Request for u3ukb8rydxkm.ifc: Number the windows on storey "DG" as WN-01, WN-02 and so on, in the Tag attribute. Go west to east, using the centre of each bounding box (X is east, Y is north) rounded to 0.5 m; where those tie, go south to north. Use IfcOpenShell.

First a look at what the model holds.

```python
import ifcopenshell
import ifcopenshell.util.element
import ifcopenshell.util.placement

model = ifcopenshell.open("u3ukb8rydxkm.ifc")
print(model.schema)
storey = next(s for s in model.by_type("IfcBuildingStorey") if s.Name == "DG")
windows = [e for e in ifcopenshell.util.element.get_decomposition(storey) if e.is_a("IfcWindow")]
for e in sorted(windows, key=lambda e: e.id()):
    origin = ifcopenshell.util.placement.get_local_placement(e.ObjectPlacement)[:3, 3]
    print(e.id(), e.Tag, e.Name, origin.round(2) + 0.0, sep=" | ")
```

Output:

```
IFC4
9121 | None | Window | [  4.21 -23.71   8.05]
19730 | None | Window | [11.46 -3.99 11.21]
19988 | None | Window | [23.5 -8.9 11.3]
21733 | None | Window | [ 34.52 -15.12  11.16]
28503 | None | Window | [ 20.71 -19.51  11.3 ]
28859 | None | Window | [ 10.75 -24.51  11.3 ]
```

```python
import ifcopenshell
import ifcopenshell.geom
import ifcopenshell.util.element
import ifcopenshell.util.shape

model = ifcopenshell.open("u3ukb8rydxkm.ifc")
settings = ifcopenshell.geom.settings()
settings.set("use-world-coords", True)


def centre(element):
    shape = ifcopenshell.geom.create_shape(settings, element)
    return ifcopenshell.util.shape.get_bbox_centroid(shape.geometry)


storey = next(s for s in model.by_type("IfcBuildingStorey") if s.Name == "DG")
windows = [e for e in ifcopenshell.util.element.get_decomposition(storey) if e.is_a("IfcWindow")]

# Insertion points can sit at a corner or the storey origin, so sort by the geometry (in metres).
centres = {e: centre(e) for e in windows}
windows.sort(key=lambda e: (round(centres[e][0] / 0.5), centres[e][1]))

for i, e in enumerate(windows, start=1):
    number = f"WN-{i:02d}"
    e.Tag = number
    print(e.id(), number)

model.write("u3ukb8rydxkm_updated.ifc")
```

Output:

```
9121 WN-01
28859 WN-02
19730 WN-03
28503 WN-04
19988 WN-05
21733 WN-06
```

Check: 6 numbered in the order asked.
